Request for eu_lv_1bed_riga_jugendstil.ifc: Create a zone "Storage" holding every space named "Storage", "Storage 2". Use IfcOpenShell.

First a look at what the model holds.

```python
import ifcopenshell

model = ifcopenshell.open("eu_lv_1bed_riga_jugendstil.ifc")
print(model.schema)
seen = {}
for space in model.by_type("IfcSpace"):
    seen[space.LongName] = seen.get(space.LongName, 0) + 1
for name, count in sorted(seen.items(), key=str):
    print(count, "x", name)
print("zones:", [z.Name for z in model.by_type("IfcZone")][:20])
```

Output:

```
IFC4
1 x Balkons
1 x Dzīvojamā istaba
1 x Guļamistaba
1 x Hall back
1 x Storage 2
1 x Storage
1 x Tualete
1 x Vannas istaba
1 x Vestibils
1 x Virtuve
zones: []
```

```python
import ifcopenshell
import ifcopenshell.api.group
import ifcopenshell.api.root

model = ifcopenshell.open("eu_lv_1bed_riga_jugendstil.ifc")

names = {"Storage", "Storage 2"}
spaces = [s for s in model.by_type("IfcSpace") if s.LongName in names]

zone = ifcopenshell.api.root.create_entity(model, ifc_class="IfcZone", name="Storage")
ifcopenshell.api.group.assign_group(model, products=spaces, group=zone)
print(len(spaces), "spaces in", zone.Name)

model.write("eu_lv_1bed_riga_jugendstil_v2.ifc")
```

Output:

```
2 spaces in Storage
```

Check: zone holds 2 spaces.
